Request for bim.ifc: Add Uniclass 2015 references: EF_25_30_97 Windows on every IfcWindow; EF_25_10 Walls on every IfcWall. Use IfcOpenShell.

First a look at what the model holds.

```python
import ifcopenshell

model = ifcopenshell.open("bim.ifc")
print(model.schema)
print("classifications:", [c.Name for c in model.by_type("IfcClassification")])
for ifc_class in ("IfcDoor", "IfcRoof", "IfcStair", "IfcWall", "IfcWindow"):
    print(ifc_class, len(model.by_type(ifc_class)))
```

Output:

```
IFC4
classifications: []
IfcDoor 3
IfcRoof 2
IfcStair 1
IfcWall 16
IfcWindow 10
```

```python
import ifcopenshell
import ifcopenshell.api.classification

model = ifcopenshell.open("bim.ifc")

system = ifcopenshell.api.classification.add_classification(model, classification="Uniclass 2015")

codes = {
    "IfcWindow": ("EF_25_30_97", "Windows"),
    "IfcWall": ("EF_25_10", "Walls"),
}
for ifc_class, (code, name) in codes.items():
    products = model.by_type(ifc_class)
    ifcopenshell.api.classification.add_reference(
        model, products=products, classification=system, identification=code, name=name
    )
    print(code, len(products))

model.write("bim_edited.ifc")
```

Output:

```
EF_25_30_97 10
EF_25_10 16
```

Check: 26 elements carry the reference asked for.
